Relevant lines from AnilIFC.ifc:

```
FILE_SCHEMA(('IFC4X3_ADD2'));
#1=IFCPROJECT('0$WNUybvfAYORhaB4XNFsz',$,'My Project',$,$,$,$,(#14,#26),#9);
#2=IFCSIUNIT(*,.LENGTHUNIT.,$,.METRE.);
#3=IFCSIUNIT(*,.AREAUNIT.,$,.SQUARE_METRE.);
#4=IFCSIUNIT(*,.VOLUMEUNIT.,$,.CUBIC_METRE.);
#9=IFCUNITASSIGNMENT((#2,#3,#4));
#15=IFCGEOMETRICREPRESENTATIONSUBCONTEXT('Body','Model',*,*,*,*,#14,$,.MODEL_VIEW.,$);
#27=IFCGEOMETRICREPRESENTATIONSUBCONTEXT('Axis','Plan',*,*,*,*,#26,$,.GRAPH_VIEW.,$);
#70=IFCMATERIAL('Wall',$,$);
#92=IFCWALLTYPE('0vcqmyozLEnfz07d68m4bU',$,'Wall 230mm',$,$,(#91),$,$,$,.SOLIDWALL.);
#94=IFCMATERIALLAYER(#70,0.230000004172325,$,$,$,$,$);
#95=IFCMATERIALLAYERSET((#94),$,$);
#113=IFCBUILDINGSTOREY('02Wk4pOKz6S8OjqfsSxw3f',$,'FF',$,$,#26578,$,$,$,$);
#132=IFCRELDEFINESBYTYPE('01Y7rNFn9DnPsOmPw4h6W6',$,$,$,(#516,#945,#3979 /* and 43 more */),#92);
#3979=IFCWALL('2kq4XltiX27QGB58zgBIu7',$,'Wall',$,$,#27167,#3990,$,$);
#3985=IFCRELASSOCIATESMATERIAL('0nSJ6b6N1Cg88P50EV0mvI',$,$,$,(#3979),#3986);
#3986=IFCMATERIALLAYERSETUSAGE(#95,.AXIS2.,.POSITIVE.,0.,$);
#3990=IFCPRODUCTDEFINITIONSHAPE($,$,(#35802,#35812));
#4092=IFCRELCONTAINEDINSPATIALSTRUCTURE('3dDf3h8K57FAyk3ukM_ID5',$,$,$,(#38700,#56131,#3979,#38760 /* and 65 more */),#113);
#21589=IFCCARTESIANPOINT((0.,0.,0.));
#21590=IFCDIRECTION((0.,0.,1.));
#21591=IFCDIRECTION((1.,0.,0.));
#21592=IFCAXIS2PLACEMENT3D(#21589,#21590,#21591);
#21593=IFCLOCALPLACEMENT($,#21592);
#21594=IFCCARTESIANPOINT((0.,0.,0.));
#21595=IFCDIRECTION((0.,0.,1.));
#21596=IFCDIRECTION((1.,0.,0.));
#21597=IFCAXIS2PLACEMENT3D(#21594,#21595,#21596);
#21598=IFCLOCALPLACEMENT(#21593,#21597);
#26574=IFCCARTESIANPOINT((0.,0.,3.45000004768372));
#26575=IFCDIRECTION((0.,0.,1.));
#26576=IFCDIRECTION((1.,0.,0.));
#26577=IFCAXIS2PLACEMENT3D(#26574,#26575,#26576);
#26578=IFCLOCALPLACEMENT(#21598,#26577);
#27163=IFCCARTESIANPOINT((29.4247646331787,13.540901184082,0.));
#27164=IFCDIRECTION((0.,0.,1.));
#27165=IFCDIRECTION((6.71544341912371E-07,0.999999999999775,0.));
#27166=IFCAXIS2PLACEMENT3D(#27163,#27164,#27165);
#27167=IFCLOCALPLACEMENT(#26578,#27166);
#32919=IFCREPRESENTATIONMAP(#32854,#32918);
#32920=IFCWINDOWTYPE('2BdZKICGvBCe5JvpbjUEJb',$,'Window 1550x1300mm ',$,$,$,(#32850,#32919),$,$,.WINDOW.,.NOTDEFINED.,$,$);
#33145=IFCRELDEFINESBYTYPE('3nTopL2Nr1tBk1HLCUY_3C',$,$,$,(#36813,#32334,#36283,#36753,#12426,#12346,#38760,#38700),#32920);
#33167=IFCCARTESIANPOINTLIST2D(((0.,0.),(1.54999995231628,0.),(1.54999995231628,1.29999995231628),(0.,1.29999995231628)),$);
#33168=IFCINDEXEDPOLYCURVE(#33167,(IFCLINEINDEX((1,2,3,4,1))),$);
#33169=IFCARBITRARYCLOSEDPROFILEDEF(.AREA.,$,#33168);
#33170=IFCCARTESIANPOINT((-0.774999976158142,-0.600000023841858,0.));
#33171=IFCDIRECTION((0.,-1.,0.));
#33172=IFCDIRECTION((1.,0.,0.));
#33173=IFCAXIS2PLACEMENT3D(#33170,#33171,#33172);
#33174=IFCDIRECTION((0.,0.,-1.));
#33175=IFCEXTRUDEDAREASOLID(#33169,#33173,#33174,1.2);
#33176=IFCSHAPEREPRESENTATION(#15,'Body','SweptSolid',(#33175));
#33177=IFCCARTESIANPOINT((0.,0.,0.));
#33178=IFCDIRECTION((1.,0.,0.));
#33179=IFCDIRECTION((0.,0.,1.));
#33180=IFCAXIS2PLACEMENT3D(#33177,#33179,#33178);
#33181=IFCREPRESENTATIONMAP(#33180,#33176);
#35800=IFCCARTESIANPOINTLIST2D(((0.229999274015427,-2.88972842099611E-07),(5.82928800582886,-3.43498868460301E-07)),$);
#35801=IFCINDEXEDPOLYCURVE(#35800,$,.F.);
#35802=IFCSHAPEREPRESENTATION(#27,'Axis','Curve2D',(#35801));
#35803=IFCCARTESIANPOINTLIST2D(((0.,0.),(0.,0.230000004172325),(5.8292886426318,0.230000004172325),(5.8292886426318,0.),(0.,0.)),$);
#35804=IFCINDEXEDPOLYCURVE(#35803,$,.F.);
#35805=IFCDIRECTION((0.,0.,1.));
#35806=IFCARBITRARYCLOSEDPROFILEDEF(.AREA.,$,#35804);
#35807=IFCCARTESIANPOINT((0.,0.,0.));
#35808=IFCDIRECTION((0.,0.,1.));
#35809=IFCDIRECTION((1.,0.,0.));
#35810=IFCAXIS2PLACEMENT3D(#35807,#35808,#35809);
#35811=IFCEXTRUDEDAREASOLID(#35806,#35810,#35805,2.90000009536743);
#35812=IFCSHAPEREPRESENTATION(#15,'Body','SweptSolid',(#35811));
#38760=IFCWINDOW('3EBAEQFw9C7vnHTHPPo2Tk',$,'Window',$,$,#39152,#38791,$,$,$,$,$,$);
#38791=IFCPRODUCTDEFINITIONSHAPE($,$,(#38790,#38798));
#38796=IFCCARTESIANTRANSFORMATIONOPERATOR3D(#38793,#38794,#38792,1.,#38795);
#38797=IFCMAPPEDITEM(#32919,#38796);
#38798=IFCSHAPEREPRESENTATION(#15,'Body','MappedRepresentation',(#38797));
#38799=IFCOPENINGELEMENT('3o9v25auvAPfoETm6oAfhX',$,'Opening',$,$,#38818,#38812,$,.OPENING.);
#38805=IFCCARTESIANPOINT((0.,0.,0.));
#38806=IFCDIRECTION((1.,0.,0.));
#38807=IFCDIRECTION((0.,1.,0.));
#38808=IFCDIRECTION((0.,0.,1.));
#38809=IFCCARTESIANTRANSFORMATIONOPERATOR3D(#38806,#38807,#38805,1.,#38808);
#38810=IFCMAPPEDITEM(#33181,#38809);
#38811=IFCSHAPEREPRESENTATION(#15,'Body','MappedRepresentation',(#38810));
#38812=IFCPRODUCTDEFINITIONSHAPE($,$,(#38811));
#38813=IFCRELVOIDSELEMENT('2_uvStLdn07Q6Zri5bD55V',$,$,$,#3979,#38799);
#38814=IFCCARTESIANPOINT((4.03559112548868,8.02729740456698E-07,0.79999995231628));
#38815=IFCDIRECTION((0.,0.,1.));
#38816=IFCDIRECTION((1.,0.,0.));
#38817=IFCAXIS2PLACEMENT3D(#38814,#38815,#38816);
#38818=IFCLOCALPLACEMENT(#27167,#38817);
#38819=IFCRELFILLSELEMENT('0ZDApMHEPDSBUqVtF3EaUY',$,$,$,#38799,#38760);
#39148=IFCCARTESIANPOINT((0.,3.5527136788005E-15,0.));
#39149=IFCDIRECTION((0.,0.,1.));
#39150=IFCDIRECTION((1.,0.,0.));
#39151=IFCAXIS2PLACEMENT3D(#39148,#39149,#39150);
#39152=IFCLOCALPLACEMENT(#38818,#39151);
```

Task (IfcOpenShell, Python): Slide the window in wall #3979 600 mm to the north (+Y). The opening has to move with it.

```python
import ifcopenshell
import ifcopenshell.api.geometry
import ifcopenshell.util.placement

model = ifcopenshell.open("AnilIFC.ifc")

window = model.by_guid("3EBAEQFw9C7vnHTHPPo2Tk")
opening = window.FillsVoids[0].RelatingOpeningElement
wall = opening.VoidsElements[0].RelatingBuildingElement

wall_matrix = ifcopenshell.util.placement.get_local_placement(wall.ObjectPlacement)
shift = wall_matrix[:3, 0] * 0.6
before = ifcopenshell.util.placement.get_local_placement(window.ObjectPlacement)[:3, 3].copy()

# The window is placed relative to its opening, so it follows when the opening moves.
matrix = ifcopenshell.util.placement.get_local_placement(opening.ObjectPlacement)
matrix[:3, 3] += shift
ifcopenshell.api.geometry.edit_object_placement(
    model, product=opening, matrix=matrix, is_si=False, should_transform_children=True
)

after = ifcopenshell.util.placement.get_local_placement(window.ObjectPlacement)[:3, 3]
print("window moved by", (after - before).round(3) + 0.0)

model.write("AnilIFC_updated.ifc")
```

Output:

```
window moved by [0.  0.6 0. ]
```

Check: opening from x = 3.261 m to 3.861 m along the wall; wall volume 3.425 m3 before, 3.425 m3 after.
